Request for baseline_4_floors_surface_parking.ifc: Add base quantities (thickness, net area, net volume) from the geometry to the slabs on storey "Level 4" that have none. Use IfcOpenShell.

First a look at what the model holds.

```python
import ifcopenshell
import ifcopenshell.util.element
import ifcopenshell.util.unit

model = ifcopenshell.open("baseline_4_floors_surface_parking.ifc")
print(model.schema)
for unit_type in ("LENGTHUNIT", "AREAUNIT", "VOLUMEUNIT"):
    print(unit_type, ifcopenshell.util.unit.calculate_unit_scale(model, unit_type))
storey = next(s for s in model.by_type("IfcBuildingStorey") if s.Name == "Level 4")
slabs = [e for e in ifcopenshell.util.element.get_decomposition(storey) if e.is_a("IfcSlab")]
for e in sorted(slabs, key=lambda e: e.id()):
    print(e.id(), e.is_a(), e.Name, list(ifcopenshell.util.element.get_psets(e, qtos_only=True)), sep=" | ")
```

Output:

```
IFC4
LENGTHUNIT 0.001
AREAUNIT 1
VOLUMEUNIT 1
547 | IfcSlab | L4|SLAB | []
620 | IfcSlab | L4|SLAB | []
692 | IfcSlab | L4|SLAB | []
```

```python
import ifcopenshell
import ifcopenshell.api.pset
import ifcopenshell.geom
import ifcopenshell.util.element
import ifcopenshell.util.shape
import ifcopenshell.util.unit

model = ifcopenshell.open("baseline_4_floors_surface_parking.ifc")
unit_scale = ifcopenshell.util.unit.calculate_unit_scale(model)
area_scale = ifcopenshell.util.unit.calculate_unit_scale(model, "AREAUNIT")
volume_scale = ifcopenshell.util.unit.calculate_unit_scale(model, "VOLUMEUNIT")
settings = ifcopenshell.geom.settings()

storey = next(s for s in model.by_type("IfcBuildingStorey") if s.Name == "Level 4")
slabs = [e for e in ifcopenshell.util.element.get_decomposition(storey) if e.is_a("IfcSlab")]

for e in sorted(slabs, key=lambda e: e.id()):
    if ifcopenshell.util.element.get_psets(e, qtos_only=True, should_inherit=False):
        continue
    # Geometry comes back in metres, in the element's own axes.
    shape = ifcopenshell.geom.create_shape(settings, e)
    values = {
        "Width": ifcopenshell.util.shape.get_z(shape.geometry) / unit_scale,
        "NetArea": ifcopenshell.util.shape.get_footprint_area(shape.geometry) / area_scale,
        "NetVolume": ifcopenshell.util.shape.get_volume(shape.geometry) / volume_scale,
    }
    qto = ifcopenshell.api.pset.add_qto(model, product=e, name="Qto_SlabBaseQuantities")
    ifcopenshell.api.pset.edit_qto(model, qto=qto, properties=values)
    print(e.id(), {k: round(v, 3) for k, v in values.items()})

model.write("baseline_4_floors_surface_parking-out.ifc")
```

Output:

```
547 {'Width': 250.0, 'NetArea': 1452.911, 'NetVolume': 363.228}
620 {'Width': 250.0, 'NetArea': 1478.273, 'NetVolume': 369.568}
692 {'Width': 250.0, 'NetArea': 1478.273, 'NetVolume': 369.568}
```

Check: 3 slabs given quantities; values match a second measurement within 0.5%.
